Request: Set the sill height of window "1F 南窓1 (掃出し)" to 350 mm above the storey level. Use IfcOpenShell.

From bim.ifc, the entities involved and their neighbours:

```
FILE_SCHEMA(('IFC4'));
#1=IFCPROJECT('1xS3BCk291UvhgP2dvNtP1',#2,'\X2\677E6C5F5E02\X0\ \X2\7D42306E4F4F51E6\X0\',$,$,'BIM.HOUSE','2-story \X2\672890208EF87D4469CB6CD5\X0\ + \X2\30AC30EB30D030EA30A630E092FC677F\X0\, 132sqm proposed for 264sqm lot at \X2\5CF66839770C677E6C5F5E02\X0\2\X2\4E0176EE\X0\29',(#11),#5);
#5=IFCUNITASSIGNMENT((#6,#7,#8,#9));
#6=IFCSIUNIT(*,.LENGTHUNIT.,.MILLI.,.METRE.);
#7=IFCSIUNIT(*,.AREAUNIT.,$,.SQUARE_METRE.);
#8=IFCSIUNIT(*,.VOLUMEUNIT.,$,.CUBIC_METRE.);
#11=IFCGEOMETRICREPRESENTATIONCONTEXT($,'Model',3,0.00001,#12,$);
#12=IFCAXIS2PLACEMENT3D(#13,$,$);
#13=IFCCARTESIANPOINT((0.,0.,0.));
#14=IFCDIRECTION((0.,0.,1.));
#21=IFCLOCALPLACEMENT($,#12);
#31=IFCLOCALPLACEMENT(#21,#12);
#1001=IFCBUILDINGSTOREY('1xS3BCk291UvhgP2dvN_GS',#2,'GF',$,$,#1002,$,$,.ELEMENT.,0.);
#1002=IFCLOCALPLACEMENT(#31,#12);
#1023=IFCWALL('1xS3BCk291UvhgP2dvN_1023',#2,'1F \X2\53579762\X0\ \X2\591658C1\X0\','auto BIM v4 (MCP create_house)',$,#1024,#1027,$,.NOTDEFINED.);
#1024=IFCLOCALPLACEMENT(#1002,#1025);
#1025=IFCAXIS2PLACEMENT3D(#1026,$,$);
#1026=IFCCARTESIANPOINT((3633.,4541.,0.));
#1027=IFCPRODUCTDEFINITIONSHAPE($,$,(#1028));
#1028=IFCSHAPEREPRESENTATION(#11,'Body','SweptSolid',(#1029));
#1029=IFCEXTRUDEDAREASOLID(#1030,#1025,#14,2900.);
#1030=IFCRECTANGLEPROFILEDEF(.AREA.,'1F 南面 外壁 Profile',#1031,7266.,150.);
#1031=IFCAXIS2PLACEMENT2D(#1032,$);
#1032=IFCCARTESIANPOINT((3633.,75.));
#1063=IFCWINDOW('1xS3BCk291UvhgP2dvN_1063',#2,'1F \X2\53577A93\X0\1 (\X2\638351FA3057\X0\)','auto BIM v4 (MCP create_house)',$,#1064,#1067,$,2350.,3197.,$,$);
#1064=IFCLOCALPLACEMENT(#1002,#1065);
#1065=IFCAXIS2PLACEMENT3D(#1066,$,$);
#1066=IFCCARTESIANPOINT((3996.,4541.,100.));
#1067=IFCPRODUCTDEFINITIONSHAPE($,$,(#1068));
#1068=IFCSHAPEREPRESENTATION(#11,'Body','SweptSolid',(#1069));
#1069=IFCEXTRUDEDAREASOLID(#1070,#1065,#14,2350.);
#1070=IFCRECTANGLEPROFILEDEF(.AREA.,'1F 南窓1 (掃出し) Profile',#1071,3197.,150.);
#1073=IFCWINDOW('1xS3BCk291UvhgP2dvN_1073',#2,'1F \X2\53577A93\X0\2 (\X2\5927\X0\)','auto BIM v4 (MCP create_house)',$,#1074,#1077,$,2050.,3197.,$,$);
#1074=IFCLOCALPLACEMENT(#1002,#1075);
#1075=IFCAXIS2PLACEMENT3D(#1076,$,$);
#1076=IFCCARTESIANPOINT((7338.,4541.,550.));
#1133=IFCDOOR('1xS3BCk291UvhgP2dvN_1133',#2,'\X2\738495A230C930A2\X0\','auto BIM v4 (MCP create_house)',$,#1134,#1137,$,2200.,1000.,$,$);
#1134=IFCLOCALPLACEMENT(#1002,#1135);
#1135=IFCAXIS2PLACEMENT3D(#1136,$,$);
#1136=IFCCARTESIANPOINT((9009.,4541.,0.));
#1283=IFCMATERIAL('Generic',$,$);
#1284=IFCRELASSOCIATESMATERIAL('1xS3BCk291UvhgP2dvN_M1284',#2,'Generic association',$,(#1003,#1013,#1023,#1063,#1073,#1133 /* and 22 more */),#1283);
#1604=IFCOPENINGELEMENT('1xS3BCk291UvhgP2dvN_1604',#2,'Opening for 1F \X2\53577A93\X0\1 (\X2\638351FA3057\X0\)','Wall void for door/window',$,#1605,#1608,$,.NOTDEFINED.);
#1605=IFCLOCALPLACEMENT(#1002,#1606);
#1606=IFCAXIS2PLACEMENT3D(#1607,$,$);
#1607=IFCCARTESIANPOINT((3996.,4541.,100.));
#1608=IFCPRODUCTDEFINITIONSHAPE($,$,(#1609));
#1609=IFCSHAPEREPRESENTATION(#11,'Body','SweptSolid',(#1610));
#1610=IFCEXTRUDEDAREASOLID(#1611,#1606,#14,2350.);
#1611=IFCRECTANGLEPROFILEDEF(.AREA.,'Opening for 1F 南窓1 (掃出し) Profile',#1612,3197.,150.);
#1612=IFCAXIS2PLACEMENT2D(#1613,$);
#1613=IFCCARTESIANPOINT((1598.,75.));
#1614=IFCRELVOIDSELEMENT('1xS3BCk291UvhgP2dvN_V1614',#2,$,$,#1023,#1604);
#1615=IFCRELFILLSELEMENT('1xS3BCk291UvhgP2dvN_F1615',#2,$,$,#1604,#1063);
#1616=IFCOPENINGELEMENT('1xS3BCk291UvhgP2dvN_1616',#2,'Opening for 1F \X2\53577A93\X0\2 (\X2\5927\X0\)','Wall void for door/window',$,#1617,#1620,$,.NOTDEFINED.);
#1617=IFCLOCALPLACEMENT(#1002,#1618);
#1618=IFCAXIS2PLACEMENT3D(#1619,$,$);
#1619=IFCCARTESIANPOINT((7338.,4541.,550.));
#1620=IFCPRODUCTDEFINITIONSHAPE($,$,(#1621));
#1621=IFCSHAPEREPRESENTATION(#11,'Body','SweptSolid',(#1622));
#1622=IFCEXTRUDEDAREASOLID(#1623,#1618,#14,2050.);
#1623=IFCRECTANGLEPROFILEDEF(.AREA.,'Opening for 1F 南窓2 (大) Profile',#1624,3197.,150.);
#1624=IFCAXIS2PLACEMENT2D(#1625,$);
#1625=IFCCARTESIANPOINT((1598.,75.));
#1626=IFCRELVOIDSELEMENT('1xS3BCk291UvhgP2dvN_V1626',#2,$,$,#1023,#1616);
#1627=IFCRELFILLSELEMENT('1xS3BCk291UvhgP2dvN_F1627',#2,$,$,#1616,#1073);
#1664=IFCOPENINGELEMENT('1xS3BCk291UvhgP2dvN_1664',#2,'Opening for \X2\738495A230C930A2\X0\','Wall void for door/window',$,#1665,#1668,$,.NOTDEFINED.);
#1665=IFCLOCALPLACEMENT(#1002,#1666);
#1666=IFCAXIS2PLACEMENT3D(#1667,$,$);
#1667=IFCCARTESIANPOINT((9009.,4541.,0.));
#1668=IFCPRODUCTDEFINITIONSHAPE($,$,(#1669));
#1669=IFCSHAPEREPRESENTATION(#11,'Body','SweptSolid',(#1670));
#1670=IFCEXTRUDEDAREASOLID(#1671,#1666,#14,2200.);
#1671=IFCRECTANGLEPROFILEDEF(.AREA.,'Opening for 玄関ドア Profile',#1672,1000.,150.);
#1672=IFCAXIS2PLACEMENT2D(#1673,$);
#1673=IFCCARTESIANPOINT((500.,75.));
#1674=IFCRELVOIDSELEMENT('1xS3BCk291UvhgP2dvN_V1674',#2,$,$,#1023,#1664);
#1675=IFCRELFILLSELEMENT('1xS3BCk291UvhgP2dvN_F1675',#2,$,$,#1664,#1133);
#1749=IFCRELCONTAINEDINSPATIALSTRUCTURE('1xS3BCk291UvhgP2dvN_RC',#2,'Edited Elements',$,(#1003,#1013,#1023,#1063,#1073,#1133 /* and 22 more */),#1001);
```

```python
import numpy as np
import ifcopenshell
import ifcopenshell.api.geometry
import ifcopenshell.geom
import ifcopenshell.util.element
import ifcopenshell.util.placement
import ifcopenshell.util.shape
import ifcopenshell.util.unit

model = ifcopenshell.open("bim.ifc")
unit_scale = ifcopenshell.util.unit.calculate_unit_scale(model)

window = model.by_guid("1xS3BCk291UvhgP2dvN_1063")
opening = window.FillsVoids[0].RelatingOpeningElement
storey = ifcopenshell.util.element.get_container(window, ifc_class="IfcBuildingStorey")
level = ifcopenshell.util.placement.get_local_placement(storey.ObjectPlacement)[2, 3]

# The opening's origin need not be at the sill, so measure its lowest point.
shape = ifcopenshell.geom.create_shape(ifcopenshell.geom.settings(), opening)
bottom = ifcopenshell.util.shape.get_shape_bottom_elevation(shape, shape.geometry) / unit_scale
dz = level + 0.35 / unit_scale - bottom

shift = np.array([0.0, 0.0, dz])
# The window is not placed relative to its opening, so move both.
for product in (opening, window):
    matrix = ifcopenshell.util.placement.get_local_placement(product.ObjectPlacement)
    matrix[:3, 3] += shift
    ifcopenshell.api.geometry.edit_object_placement(model, product=product, matrix=matrix, is_si=False)

print(f"moved by {dz * unit_scale:+.3f} m")

model.write("bim_rev.ifc")
```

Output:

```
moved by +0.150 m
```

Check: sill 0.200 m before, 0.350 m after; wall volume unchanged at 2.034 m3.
